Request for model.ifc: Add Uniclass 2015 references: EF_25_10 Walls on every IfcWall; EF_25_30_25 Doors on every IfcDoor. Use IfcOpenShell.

First a look at what the model holds.

```python
import ifcopenshell

model = ifcopenshell.open("model.ifc")
print(model.schema)
print("classifications:", [c.Name for c in model.by_type("IfcClassification")])
for ifc_class in ("IfcDoor", "IfcRoof", "IfcStair", "IfcWall", "IfcWindow"):
    print(ifc_class, len(model.by_type(ifc_class)))
```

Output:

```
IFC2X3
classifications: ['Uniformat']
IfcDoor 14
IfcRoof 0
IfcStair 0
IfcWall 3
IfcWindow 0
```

```python
import ifcopenshell
import ifcopenshell.api.classification

model = ifcopenshell.open("model.ifc")

# IFC2X3 requires Source and Edition and has no link from the project to the system.
system = model.create_entity("IfcClassification", Source="NBS", Edition="2015", Name="Uniclass 2015")

codes = {
    "IfcWall": ("EF_25_10", "Walls"),
    "IfcDoor": ("EF_25_30_25", "Doors"),
}
for ifc_class, (code, name) in codes.items():
    products = model.by_type(ifc_class)
    ifcopenshell.api.classification.add_reference(
        model, products=products, classification=system, identification=code, name=name
    )
    print(code, len(products))

model.write("model_rev.ifc")
```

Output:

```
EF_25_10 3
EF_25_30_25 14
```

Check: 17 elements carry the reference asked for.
